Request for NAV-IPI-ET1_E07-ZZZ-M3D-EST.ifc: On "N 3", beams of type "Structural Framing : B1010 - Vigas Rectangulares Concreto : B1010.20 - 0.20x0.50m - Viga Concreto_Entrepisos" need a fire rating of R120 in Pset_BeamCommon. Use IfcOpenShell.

First a look at what the model holds.

```python
import ifcopenshell
import ifcopenshell.util.element

model = ifcopenshell.open("NAV-IPI-ET1_E07-ZZZ-M3D-EST.ifc")
print(model.schema)
storey = next(s for s in model.by_type("IfcBuildingStorey") if s.Name == "N 3")
beams = [e for e in ifcopenshell.util.element.get_decomposition(storey) if e.is_a("IfcBeam")]
seen = {}
for e in beams:
    element_type = ifcopenshell.util.element.get_type(e)
    key = (element_type.Name if element_type != e and element_type else None, ifcopenshell.util.element.get_pset(e, "Pset_BeamCommon", "FireRating"))
    seen[key] = seen.get(key, 0) + 1
for (name, value), count in sorted(seen.items(), key=str):
    print(count, "x", name, "|", value)
```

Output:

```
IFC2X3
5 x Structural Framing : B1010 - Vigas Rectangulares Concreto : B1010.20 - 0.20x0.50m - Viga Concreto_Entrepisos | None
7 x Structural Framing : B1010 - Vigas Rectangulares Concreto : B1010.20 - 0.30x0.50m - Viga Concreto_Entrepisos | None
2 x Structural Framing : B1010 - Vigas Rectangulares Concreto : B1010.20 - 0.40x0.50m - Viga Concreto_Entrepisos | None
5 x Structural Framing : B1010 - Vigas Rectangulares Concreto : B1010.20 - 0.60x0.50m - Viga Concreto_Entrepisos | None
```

```python
import ifcopenshell
import ifcopenshell.api.pset
import ifcopenshell.util.element

model = ifcopenshell.open("NAV-IPI-ET1_E07-ZZZ-M3D-EST.ifc")

storey = next(s for s in model.by_type("IfcBuildingStorey") if s.Name == "N 3")
beams = [e for e in ifcopenshell.util.element.get_decomposition(storey) if e.is_a("IfcBeam")]

count = 0
for e in beams:
    element_type = ifcopenshell.util.element.get_type(e)
    if element_type in (None, e) or element_type.Name != "Structural Framing : B1010 - Vigas Rectangulares Concreto : B1010.20 - 0.20x0.50m - Viga Concreto_Entrepisos":
        continue
    # add_pset returns the element's existing set when there is one.
    pset = ifcopenshell.api.pset.add_pset(model, product=e, name="Pset_BeamCommon")
    ifcopenshell.api.pset.edit_pset(model, pset=pset, properties={"FireRating": "R120"})
    count += 1

print(count, "beams updated")

model.write("NAV-IPI-ET1_E07-ZZZ-M3D-EST_updated.ifc")
```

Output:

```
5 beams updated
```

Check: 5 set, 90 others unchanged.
